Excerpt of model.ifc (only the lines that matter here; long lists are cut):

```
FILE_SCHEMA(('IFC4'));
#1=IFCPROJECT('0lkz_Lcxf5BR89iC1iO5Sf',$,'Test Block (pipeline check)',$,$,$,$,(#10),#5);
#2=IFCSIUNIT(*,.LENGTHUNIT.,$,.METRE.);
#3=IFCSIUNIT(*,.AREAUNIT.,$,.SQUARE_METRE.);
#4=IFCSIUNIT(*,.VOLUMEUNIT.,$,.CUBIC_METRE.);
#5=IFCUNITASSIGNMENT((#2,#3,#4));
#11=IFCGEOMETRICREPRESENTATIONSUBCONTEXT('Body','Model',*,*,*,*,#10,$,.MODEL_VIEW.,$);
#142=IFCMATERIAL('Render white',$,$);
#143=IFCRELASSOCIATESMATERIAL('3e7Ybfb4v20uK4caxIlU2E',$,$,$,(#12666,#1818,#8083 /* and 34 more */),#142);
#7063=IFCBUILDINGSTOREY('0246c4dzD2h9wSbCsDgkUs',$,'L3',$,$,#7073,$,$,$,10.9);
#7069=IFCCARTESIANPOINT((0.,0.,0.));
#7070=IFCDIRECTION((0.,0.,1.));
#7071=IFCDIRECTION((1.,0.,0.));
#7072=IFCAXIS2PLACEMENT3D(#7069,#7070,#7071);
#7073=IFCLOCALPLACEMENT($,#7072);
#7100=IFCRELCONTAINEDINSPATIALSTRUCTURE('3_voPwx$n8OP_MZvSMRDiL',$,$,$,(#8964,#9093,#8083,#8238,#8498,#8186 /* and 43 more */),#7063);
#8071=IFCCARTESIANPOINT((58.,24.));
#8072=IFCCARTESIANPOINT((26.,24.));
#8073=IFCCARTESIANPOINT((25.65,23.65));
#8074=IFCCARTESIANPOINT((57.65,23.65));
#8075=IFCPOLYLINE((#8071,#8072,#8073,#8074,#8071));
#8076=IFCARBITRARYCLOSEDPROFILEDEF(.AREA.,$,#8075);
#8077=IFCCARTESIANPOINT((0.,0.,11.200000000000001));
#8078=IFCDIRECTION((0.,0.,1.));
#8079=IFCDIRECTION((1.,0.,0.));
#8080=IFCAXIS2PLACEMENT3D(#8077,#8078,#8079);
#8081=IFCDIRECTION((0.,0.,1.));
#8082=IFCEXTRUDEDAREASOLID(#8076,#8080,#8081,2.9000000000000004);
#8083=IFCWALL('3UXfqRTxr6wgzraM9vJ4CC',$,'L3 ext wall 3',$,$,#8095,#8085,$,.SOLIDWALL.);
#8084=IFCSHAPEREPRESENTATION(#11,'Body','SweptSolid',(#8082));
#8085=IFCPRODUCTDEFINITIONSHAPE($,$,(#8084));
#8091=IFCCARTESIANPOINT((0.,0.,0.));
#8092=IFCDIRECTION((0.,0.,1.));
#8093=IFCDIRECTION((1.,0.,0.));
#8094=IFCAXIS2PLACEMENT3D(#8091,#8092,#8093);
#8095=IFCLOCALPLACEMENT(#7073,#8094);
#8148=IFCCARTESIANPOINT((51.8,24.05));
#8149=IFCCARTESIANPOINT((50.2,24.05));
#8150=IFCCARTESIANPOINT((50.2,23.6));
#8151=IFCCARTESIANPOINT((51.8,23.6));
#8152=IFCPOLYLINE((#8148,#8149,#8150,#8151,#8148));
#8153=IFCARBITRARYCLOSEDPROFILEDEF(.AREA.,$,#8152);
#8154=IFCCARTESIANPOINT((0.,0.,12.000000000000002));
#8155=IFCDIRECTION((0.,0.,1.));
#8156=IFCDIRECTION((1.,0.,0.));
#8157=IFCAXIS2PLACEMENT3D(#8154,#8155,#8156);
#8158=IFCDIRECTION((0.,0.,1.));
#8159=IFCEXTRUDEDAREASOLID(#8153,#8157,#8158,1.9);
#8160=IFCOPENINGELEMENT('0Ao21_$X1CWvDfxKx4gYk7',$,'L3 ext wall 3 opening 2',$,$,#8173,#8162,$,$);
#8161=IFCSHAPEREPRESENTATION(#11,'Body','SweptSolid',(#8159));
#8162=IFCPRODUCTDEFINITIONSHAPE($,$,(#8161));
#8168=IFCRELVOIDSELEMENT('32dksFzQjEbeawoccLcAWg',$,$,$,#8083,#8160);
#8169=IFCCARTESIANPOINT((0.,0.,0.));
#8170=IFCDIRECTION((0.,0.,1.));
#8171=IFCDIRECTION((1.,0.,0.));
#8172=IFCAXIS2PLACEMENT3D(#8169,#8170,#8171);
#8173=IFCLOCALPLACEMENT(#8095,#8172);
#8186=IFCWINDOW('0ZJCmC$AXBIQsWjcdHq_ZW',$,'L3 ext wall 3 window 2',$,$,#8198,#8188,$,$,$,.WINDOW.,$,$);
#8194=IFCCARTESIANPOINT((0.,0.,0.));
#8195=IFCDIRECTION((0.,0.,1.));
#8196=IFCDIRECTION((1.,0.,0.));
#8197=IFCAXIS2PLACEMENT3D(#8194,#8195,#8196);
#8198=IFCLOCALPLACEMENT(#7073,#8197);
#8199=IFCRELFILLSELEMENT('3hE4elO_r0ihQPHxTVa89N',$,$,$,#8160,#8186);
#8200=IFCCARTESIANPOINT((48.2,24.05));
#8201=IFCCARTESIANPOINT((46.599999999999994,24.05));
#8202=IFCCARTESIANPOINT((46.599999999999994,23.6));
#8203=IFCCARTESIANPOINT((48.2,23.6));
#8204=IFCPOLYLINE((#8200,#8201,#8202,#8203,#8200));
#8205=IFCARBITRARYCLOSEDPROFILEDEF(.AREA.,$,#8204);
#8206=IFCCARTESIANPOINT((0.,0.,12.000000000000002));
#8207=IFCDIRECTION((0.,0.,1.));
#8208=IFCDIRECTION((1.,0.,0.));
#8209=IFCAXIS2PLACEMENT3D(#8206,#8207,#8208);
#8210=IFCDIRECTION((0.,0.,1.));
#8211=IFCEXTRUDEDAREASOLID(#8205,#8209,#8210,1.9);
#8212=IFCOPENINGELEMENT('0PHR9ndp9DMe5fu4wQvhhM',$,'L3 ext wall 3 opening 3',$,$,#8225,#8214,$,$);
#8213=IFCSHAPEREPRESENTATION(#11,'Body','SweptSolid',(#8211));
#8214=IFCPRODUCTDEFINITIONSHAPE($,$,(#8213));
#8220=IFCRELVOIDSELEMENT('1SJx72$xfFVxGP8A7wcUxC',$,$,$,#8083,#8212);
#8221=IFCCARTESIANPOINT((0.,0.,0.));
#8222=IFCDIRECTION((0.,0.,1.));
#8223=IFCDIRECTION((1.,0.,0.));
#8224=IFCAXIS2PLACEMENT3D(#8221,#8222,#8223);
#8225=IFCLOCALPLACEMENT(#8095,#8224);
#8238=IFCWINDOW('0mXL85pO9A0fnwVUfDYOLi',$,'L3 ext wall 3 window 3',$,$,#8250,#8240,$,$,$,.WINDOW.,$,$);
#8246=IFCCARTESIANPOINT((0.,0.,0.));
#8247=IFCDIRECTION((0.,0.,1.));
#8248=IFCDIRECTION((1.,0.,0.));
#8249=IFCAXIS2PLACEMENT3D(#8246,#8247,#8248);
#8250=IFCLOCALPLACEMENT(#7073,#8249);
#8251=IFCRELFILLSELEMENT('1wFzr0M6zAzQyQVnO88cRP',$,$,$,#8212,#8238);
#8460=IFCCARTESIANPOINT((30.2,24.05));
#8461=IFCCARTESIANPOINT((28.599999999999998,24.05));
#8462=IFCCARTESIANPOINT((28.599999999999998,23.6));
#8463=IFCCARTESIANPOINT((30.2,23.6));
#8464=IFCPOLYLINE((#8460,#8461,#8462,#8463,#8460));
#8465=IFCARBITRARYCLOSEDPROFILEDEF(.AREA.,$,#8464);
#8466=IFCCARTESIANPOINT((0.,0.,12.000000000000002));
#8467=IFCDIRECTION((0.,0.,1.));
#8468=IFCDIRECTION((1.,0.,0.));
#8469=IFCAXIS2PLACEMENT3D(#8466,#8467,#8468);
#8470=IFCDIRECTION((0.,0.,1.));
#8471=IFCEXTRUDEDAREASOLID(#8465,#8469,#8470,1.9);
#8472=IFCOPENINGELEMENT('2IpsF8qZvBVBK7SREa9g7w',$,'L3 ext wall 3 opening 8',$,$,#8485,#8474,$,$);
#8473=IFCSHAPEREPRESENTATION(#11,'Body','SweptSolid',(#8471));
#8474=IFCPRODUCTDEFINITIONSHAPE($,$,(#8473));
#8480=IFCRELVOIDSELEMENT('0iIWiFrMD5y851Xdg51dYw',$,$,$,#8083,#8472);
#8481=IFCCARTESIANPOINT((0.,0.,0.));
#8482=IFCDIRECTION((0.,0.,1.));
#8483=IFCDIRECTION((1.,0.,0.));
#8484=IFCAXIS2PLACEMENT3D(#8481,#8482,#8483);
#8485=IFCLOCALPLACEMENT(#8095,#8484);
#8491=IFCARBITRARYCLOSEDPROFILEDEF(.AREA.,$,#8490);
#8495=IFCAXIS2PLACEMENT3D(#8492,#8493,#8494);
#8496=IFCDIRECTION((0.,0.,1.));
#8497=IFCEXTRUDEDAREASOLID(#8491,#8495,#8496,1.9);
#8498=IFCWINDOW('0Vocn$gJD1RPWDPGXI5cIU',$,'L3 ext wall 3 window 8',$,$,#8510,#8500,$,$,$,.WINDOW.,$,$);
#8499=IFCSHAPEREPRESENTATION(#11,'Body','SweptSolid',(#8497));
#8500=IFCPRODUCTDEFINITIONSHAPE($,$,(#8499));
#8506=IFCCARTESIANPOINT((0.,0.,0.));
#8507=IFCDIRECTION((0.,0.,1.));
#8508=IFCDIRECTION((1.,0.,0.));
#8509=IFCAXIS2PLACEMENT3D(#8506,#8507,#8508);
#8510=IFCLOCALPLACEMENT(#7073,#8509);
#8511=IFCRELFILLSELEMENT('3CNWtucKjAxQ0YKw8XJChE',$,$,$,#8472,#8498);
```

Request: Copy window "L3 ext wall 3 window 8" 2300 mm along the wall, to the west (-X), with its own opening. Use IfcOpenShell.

```python
import ifcopenshell
import ifcopenshell.api.feature
import ifcopenshell.api.geometry
import ifcopenshell.api.root
import ifcopenshell.geom
import ifcopenshell.util.element
import ifcopenshell.util.placement
import ifcopenshell.util.shape
import ifcopenshell.util.unit

model = ifcopenshell.open("model.ifc")
unit_scale = ifcopenshell.util.unit.calculate_unit_scale(model)
settings = ifcopenshell.geom.settings()


def volume(element):
    """Net volume in cubic metres, openings subtracted."""
    shape = ifcopenshell.geom.create_shape(settings, element)
    return ifcopenshell.util.shape.get_volume(shape.geometry)


window = model.by_guid("0Vocn$gJD1RPWDPGXI5cIU")
opening = window.FillsVoids[0].RelatingOpeningElement
wall = opening.VoidsElements[0].RelatingBuildingElement
before = volume(wall)
shift = ifcopenshell.util.placement.get_local_placement(wall.ObjectPlacement)[:3, 0] * -2.3 / unit_scale

# copy_class copies the void relationship, type, container and properties, but no geometry.
new_opening = ifcopenshell.api.root.copy_class(model, product=opening)
new_opening.Representation = ifcopenshell.util.element.copy_deep(
    model, opening.Representation, exclude=["IfcGeometricRepresentationContext", "IfcRepresentationMap"]
)
new_window = ifcopenshell.api.root.copy_class(model, product=window)
new_window.Representation = ifcopenshell.util.element.copy_deep(
    model, window.Representation, exclude=["IfcGeometricRepresentationContext", "IfcRepresentationMap"]
)
ifcopenshell.api.feature.add_filling(model, opening=new_opening, element=new_window)

for old, new in ((opening, new_opening), (window, new_window)):
    matrix = ifcopenshell.util.placement.get_local_placement(old.ObjectPlacement)
    matrix[:3, 3] += shift
    ifcopenshell.api.geometry.edit_object_placement(model, product=new, matrix=matrix, is_si=False)

after = volume(wall)

print(f"wall volume {before:.3f} -> {after:.3f} m3")

model.write("model_updated.ifc")
```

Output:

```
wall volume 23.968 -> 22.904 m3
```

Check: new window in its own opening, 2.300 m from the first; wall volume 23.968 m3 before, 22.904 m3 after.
